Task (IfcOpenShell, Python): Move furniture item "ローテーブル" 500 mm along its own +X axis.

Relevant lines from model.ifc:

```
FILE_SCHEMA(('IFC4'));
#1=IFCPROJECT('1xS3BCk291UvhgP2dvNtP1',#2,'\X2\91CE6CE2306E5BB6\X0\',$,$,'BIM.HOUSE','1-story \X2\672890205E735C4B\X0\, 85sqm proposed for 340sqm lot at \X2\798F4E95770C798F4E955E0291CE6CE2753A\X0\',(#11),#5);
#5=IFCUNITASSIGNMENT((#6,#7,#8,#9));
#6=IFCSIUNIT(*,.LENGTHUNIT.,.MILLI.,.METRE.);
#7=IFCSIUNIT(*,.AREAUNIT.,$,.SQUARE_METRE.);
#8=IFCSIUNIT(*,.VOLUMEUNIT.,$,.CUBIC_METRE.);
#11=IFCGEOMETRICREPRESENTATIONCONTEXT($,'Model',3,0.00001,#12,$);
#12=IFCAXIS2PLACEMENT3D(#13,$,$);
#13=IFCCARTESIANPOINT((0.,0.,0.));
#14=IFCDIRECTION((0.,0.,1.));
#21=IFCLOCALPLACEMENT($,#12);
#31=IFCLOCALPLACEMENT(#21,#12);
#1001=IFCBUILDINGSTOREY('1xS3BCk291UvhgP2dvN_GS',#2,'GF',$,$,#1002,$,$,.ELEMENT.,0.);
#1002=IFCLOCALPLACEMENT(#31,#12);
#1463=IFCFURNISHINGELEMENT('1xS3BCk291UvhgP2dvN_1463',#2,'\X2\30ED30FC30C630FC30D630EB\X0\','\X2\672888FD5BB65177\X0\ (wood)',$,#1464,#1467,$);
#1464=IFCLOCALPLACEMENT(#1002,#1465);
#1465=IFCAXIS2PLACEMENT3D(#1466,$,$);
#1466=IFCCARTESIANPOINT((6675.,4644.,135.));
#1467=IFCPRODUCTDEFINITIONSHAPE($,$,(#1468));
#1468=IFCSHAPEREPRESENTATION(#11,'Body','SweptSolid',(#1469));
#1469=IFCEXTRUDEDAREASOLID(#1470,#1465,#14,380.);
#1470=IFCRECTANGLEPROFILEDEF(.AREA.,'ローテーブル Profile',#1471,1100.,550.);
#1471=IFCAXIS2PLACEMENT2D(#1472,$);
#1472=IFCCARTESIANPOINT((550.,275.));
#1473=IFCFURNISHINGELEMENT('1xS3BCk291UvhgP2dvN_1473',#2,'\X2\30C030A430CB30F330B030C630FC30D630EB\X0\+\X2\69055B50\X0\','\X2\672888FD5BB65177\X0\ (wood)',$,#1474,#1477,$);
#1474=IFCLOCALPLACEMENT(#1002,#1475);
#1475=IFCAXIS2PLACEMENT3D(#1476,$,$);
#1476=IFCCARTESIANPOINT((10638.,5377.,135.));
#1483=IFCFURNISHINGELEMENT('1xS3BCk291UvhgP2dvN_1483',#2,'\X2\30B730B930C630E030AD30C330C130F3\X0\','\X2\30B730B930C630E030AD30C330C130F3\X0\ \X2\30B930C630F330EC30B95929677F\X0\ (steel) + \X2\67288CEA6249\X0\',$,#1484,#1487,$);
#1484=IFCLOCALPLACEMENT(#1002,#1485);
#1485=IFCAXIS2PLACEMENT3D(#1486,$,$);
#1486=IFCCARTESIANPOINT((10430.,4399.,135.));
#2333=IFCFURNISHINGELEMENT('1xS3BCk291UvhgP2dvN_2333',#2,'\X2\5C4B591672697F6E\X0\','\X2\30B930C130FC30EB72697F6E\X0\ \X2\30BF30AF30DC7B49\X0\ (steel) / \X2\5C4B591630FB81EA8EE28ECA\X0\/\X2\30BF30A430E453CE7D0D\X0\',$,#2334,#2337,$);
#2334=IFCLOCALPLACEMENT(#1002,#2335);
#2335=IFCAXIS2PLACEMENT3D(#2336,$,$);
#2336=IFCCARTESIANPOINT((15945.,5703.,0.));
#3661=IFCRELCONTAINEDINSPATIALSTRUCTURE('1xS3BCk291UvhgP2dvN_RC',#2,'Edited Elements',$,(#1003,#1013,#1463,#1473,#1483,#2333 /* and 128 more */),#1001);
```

```python
import ifcopenshell
import ifcopenshell.api.geometry
import ifcopenshell.util.placement

model = ifcopenshell.open("model.ifc")

item = model.by_guid("1xS3BCk291UvhgP2dvN_1463")
matrix = ifcopenshell.util.placement.get_local_placement(item.ObjectPlacement)
matrix[:3, 3] += matrix[:3, 0] * 500.0
ifcopenshell.api.geometry.edit_object_placement(model, product=item, matrix=matrix, is_si=False)

print(ifcopenshell.util.placement.get_local_placement(item.ObjectPlacement).round(3) + 0.0)

model.write("model-out.ifc")
```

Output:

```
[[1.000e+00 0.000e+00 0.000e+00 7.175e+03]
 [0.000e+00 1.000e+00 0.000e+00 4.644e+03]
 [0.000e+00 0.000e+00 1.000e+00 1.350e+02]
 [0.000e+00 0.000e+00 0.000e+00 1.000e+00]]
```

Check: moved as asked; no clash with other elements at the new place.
